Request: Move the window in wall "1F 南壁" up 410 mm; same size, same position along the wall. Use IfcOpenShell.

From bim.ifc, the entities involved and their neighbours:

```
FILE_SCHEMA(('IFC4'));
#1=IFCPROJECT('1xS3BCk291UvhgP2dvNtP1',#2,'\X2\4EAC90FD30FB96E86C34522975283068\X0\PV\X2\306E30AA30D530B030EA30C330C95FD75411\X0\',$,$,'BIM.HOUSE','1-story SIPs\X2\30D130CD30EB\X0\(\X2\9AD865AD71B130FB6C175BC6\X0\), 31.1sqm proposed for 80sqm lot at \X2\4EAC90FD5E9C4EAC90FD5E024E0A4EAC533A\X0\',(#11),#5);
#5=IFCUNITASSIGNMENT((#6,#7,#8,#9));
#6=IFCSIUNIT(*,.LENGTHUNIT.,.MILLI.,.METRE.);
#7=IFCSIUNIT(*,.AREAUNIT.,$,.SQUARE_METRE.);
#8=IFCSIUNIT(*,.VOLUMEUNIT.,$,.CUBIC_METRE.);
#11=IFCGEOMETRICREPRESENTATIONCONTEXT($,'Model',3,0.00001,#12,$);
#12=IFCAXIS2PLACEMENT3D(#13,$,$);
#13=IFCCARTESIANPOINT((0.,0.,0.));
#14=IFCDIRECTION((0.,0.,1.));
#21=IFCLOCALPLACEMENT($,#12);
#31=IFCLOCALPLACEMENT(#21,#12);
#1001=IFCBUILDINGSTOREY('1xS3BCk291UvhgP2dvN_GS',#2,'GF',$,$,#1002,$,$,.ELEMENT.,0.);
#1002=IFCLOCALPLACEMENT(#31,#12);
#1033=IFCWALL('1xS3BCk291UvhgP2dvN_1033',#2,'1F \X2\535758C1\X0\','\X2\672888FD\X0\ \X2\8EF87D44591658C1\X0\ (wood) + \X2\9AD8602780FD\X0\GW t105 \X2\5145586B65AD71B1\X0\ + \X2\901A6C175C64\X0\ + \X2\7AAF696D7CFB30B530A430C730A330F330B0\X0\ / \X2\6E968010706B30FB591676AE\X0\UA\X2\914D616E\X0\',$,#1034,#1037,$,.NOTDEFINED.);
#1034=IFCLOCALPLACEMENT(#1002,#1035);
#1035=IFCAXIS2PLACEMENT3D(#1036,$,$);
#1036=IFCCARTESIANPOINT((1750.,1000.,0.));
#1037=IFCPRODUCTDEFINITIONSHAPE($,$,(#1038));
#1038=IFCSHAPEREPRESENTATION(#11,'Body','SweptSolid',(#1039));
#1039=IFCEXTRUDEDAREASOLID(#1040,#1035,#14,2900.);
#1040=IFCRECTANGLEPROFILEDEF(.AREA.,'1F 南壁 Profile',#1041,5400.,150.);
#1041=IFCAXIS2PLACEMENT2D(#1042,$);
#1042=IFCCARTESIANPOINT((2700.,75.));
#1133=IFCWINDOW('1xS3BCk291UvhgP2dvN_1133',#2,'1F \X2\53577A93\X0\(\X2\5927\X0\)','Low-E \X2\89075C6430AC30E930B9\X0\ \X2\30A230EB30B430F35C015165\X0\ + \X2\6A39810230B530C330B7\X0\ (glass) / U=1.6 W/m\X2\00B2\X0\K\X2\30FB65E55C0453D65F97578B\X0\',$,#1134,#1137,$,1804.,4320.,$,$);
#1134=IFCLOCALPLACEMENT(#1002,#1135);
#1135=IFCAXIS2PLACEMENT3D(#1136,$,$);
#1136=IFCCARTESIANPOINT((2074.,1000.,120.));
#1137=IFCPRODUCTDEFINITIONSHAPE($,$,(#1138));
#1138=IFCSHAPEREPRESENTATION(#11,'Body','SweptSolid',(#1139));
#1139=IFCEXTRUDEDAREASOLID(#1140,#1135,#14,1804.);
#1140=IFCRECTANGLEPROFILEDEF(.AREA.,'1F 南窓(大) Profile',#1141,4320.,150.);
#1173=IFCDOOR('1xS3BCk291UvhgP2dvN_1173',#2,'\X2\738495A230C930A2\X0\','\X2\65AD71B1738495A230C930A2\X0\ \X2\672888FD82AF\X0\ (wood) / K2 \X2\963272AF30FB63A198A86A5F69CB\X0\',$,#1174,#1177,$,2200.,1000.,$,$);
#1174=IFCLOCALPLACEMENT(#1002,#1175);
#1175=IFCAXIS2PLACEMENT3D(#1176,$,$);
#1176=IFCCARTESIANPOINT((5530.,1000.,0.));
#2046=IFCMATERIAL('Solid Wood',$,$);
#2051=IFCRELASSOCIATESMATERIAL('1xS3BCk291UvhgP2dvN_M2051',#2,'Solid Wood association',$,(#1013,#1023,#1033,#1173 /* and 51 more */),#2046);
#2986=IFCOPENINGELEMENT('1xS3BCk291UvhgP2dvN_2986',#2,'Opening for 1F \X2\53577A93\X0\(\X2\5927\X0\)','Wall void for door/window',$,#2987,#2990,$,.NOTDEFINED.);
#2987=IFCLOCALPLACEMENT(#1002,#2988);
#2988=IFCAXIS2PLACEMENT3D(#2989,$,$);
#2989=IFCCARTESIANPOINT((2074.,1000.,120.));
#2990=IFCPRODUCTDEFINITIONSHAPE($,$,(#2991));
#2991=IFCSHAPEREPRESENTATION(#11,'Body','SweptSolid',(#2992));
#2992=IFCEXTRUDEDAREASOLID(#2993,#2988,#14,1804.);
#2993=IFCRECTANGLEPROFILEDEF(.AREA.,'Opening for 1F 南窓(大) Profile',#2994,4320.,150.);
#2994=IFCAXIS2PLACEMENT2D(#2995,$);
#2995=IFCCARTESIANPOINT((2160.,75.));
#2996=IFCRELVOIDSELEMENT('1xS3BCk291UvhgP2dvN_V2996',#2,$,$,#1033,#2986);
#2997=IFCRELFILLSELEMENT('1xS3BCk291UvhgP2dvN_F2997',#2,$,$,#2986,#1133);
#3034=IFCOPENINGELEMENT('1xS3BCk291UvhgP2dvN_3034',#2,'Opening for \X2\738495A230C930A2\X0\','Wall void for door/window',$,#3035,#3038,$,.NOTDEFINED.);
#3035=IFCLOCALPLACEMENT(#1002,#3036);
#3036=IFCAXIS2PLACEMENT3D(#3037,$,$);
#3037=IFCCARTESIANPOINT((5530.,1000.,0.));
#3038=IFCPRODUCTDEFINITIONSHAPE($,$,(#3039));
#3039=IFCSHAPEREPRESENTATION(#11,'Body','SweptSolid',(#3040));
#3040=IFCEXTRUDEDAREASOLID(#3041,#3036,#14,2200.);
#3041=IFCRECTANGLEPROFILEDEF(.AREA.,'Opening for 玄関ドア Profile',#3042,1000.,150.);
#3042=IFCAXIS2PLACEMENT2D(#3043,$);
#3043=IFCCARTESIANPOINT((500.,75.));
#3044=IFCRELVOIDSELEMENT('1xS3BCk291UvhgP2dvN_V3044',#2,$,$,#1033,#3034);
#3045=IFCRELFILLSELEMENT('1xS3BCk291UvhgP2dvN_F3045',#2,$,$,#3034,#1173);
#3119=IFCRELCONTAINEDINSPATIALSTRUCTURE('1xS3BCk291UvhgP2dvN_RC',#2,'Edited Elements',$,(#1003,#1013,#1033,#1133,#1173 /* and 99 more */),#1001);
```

```python
import numpy as np
import ifcopenshell
import ifcopenshell.api.geometry
import ifcopenshell.util.placement
import ifcopenshell.util.unit

model = ifcopenshell.open("bim.ifc")
unit_scale = ifcopenshell.util.unit.calculate_unit_scale(model)

window = model.by_guid("1xS3BCk291UvhgP2dvN_1133")
opening = window.FillsVoids[0].RelatingOpeningElement
dz = 410.0

shift = np.array([0.0, 0.0, dz])
# The window is not placed relative to its opening, so move both.
for product in (opening, window):
    matrix = ifcopenshell.util.placement.get_local_placement(product.ObjectPlacement)
    matrix[:3, 3] += shift
    ifcopenshell.api.geometry.edit_object_placement(model, product=product, matrix=matrix, is_si=False)

print(f"moved by {dz * unit_scale:+.3f} m")

model.write("bim-out.ifc")
```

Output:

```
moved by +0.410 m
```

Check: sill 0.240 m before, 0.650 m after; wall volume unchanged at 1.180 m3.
